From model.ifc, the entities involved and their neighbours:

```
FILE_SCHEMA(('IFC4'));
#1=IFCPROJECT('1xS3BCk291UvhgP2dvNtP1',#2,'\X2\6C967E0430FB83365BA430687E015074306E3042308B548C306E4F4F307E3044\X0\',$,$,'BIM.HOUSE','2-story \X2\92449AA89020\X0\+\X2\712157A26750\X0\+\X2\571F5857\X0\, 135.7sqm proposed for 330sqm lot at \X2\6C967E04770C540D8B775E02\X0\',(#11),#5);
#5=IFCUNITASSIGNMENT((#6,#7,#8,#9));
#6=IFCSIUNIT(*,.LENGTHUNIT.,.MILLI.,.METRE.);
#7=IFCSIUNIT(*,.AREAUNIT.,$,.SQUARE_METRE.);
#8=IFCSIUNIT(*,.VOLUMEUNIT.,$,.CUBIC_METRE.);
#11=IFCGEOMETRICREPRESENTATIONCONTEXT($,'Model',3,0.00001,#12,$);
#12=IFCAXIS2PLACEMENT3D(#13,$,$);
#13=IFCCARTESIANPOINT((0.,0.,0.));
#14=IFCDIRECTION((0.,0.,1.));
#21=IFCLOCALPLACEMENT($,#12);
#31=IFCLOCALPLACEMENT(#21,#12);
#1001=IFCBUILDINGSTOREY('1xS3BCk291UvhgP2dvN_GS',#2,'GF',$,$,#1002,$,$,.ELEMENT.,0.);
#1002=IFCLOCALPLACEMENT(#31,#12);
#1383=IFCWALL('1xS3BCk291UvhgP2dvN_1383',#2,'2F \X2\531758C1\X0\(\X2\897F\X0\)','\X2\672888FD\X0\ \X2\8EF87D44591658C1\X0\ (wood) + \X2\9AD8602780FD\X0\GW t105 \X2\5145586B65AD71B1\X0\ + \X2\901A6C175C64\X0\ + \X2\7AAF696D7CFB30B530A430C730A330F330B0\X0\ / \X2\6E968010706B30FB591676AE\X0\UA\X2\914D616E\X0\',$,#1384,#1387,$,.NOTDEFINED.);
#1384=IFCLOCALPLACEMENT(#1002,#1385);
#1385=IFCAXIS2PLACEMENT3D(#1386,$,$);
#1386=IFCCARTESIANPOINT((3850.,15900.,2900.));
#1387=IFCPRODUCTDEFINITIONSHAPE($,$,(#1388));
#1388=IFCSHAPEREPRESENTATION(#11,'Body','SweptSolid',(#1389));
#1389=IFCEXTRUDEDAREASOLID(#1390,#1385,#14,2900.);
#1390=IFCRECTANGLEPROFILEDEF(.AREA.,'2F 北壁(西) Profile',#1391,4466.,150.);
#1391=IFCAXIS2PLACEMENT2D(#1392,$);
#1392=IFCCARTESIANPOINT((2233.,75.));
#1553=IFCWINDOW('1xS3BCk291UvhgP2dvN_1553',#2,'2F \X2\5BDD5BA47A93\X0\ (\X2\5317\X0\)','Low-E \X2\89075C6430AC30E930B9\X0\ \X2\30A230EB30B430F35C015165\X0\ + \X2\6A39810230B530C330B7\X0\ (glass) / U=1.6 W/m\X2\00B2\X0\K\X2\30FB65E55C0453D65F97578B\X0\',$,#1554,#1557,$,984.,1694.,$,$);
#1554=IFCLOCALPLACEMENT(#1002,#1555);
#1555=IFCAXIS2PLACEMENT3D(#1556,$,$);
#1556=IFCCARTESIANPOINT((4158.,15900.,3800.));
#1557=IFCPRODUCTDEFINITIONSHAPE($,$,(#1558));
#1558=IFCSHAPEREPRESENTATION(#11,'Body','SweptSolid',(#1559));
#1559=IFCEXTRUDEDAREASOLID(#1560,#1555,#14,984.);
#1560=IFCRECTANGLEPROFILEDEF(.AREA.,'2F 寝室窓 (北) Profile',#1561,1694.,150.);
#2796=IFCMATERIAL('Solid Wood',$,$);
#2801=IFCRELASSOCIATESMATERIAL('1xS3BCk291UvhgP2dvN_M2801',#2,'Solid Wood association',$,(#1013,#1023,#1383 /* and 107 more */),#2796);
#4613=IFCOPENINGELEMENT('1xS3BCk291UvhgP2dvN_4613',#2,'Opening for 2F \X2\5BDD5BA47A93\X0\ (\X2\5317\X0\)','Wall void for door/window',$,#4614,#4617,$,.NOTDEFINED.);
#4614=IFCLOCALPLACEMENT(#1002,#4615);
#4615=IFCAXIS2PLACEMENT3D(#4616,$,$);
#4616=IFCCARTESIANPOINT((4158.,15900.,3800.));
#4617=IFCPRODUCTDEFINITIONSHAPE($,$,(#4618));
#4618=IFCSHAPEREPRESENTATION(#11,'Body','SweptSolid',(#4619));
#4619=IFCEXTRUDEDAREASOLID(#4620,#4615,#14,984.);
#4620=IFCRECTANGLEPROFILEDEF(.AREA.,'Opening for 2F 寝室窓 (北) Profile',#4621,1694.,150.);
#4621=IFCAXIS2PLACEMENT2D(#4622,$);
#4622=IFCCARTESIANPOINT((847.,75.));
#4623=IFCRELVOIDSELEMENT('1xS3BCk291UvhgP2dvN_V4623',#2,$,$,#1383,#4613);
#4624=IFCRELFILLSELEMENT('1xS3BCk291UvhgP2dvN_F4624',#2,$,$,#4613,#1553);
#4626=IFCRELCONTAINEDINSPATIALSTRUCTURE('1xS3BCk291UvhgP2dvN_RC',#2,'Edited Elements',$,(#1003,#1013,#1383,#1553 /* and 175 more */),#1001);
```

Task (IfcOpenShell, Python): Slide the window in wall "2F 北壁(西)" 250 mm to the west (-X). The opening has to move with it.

```python
import ifcopenshell
import ifcopenshell.api.geometry
import ifcopenshell.util.placement

model = ifcopenshell.open("model.ifc")

window = model.by_id(1553)
opening = window.FillsVoids[0].RelatingOpeningElement
wall = opening.VoidsElements[0].RelatingBuildingElement

wall_matrix = ifcopenshell.util.placement.get_local_placement(wall.ObjectPlacement)
shift = wall_matrix[:3, 0] * -250.0
before = ifcopenshell.util.placement.get_local_placement(window.ObjectPlacement)[:3, 3].copy()

# The window is not placed relative to its opening, so move both.
for product in (opening, window):
    matrix = ifcopenshell.util.placement.get_local_placement(product.ObjectPlacement)
    matrix[:3, 3] += shift
    ifcopenshell.api.geometry.edit_object_placement(model, product=product, matrix=matrix, is_si=False)

after = ifcopenshell.util.placement.get_local_placement(window.ObjectPlacement)[:3, 3]
print("window moved by", (after - before).round(3) + 0.0)

model.write("model_edited.ifc")
```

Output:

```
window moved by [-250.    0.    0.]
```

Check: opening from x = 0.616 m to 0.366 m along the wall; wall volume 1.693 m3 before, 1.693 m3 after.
